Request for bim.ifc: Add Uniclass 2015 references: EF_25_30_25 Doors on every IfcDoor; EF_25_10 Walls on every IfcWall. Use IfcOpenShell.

First a look at what the model holds.

```python
import ifcopenshell

model = ifcopenshell.open("bim.ifc")
print(model.schema)
print("classifications:", [c.Name for c in model.by_type("IfcClassification")])
for ifc_class in ("IfcDoor", "IfcRoof", "IfcStair", "IfcWall", "IfcWindow"):
    print(ifc_class, len(model.by_type(ifc_class)))
```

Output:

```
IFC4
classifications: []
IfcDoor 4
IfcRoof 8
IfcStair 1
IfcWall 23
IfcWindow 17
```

```python
import ifcopenshell
import ifcopenshell.api.classification

model = ifcopenshell.open("bim.ifc")

system = ifcopenshell.api.classification.add_classification(model, classification="Uniclass 2015")

codes = {
    "IfcDoor": ("EF_25_30_25", "Doors"),
    "IfcWall": ("EF_25_10", "Walls"),
}
for ifc_class, (code, name) in codes.items():
    products = model.by_type(ifc_class)
    ifcopenshell.api.classification.add_reference(
        model, products=products, classification=system, identification=code, name=name
    )
    print(code, len(products))

model.write("bim_updated.ifc")
```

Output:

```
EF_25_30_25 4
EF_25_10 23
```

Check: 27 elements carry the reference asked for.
